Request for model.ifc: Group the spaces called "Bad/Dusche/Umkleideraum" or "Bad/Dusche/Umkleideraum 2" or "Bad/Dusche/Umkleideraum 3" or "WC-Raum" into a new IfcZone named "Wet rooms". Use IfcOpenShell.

First a look at what the model holds.

```python
import ifcopenshell

model = ifcopenshell.open("model.ifc")
print(model.schema)
seen = {}
for space in model.by_type("IfcSpace"):
    seen[space.Name] = seen.get(space.Name, 0) + 1
for name, count in sorted(seen.items(), key=str):
    print(count, "x", name)
print("zones:", [z.Name for z in model.by_type("IfcZone")][:20])
```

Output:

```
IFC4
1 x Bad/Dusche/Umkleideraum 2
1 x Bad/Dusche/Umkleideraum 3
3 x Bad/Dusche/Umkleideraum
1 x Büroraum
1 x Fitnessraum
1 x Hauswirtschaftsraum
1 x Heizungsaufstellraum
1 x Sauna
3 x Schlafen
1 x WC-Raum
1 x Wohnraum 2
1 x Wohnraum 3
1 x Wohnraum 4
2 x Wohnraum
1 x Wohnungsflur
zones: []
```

```python
import ifcopenshell
import ifcopenshell.api.group
import ifcopenshell.api.root

model = ifcopenshell.open("model.ifc")

names = {"Bad/Dusche/Umkleideraum", "Bad/Dusche/Umkleideraum 2", "Bad/Dusche/Umkleideraum 3", "WC-Raum"}
spaces = [s for s in model.by_type("IfcSpace") if s.Name in names]

zone = ifcopenshell.api.root.create_entity(model, ifc_class="IfcZone", name="Wet rooms")
ifcopenshell.api.group.assign_group(model, products=spaces, group=zone)
print(len(spaces), "spaces in", zone.Name)

model.write("model_v2.ifc")
```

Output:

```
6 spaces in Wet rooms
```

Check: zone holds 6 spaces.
